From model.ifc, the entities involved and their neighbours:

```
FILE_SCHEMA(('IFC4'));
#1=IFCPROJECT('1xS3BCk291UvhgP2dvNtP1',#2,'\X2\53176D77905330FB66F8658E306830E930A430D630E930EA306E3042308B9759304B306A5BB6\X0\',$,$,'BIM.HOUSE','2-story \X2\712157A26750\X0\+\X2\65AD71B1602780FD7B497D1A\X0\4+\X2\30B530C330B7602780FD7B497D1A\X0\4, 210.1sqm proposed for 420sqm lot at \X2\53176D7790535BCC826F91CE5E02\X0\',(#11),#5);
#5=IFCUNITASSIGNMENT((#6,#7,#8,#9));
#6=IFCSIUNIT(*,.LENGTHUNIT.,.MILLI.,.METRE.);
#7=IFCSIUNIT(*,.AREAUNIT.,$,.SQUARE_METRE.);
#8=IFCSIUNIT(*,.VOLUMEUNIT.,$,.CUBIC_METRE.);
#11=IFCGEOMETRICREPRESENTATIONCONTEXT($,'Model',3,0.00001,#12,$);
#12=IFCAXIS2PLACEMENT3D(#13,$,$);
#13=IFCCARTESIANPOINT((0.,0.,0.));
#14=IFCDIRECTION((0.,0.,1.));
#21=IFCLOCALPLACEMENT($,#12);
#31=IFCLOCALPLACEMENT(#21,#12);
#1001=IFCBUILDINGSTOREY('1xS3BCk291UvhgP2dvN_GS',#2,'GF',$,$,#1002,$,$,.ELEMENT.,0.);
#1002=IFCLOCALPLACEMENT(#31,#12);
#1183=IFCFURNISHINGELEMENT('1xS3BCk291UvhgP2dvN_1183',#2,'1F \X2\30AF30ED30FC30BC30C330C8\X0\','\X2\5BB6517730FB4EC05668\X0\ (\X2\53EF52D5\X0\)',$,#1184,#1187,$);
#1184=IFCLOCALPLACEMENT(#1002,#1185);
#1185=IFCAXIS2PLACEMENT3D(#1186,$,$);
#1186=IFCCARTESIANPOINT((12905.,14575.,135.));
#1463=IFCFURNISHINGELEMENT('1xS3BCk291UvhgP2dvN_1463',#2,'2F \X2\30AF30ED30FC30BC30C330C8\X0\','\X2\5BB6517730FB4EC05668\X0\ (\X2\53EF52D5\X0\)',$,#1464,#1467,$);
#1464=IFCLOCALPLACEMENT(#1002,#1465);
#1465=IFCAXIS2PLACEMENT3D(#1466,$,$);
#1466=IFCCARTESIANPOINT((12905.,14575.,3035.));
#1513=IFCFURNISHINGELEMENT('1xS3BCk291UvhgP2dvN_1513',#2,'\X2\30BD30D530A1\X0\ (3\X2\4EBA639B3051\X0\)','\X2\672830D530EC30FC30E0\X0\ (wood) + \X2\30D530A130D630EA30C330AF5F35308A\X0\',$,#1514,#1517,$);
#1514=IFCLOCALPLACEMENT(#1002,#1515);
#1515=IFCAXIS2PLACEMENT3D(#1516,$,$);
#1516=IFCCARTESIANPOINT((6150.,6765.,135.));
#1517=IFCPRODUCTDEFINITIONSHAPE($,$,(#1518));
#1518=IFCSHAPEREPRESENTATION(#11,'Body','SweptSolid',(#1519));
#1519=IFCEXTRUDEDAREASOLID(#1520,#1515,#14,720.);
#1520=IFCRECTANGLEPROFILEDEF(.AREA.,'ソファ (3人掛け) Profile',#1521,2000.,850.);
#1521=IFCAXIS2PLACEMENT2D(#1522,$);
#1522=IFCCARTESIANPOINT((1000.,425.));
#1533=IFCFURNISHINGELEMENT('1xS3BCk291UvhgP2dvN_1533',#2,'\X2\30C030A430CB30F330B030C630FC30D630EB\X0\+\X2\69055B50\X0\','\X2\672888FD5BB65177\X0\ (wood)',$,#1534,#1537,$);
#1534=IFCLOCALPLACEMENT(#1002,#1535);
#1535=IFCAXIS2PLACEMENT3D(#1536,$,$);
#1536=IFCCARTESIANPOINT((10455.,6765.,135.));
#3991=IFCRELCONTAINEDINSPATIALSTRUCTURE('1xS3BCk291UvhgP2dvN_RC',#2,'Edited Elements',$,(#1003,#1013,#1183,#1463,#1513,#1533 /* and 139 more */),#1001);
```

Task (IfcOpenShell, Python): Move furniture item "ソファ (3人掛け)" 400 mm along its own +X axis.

```python
import ifcopenshell
import ifcopenshell.api.geometry
import ifcopenshell.util.placement

model = ifcopenshell.open("model.ifc")

item = model.by_guid("1xS3BCk291UvhgP2dvN_1513")
matrix = ifcopenshell.util.placement.get_local_placement(item.ObjectPlacement)
matrix[:3, 3] += matrix[:3, 0] * 400.0
ifcopenshell.api.geometry.edit_object_placement(model, product=item, matrix=matrix, is_si=False)

print(ifcopenshell.util.placement.get_local_placement(item.ObjectPlacement).round(3) + 0.0)

model.write("model_updated.ifc")
```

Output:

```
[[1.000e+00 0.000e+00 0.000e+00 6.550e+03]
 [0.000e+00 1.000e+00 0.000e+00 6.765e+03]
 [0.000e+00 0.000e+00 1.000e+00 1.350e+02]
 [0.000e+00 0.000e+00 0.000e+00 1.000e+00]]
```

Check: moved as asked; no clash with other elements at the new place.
